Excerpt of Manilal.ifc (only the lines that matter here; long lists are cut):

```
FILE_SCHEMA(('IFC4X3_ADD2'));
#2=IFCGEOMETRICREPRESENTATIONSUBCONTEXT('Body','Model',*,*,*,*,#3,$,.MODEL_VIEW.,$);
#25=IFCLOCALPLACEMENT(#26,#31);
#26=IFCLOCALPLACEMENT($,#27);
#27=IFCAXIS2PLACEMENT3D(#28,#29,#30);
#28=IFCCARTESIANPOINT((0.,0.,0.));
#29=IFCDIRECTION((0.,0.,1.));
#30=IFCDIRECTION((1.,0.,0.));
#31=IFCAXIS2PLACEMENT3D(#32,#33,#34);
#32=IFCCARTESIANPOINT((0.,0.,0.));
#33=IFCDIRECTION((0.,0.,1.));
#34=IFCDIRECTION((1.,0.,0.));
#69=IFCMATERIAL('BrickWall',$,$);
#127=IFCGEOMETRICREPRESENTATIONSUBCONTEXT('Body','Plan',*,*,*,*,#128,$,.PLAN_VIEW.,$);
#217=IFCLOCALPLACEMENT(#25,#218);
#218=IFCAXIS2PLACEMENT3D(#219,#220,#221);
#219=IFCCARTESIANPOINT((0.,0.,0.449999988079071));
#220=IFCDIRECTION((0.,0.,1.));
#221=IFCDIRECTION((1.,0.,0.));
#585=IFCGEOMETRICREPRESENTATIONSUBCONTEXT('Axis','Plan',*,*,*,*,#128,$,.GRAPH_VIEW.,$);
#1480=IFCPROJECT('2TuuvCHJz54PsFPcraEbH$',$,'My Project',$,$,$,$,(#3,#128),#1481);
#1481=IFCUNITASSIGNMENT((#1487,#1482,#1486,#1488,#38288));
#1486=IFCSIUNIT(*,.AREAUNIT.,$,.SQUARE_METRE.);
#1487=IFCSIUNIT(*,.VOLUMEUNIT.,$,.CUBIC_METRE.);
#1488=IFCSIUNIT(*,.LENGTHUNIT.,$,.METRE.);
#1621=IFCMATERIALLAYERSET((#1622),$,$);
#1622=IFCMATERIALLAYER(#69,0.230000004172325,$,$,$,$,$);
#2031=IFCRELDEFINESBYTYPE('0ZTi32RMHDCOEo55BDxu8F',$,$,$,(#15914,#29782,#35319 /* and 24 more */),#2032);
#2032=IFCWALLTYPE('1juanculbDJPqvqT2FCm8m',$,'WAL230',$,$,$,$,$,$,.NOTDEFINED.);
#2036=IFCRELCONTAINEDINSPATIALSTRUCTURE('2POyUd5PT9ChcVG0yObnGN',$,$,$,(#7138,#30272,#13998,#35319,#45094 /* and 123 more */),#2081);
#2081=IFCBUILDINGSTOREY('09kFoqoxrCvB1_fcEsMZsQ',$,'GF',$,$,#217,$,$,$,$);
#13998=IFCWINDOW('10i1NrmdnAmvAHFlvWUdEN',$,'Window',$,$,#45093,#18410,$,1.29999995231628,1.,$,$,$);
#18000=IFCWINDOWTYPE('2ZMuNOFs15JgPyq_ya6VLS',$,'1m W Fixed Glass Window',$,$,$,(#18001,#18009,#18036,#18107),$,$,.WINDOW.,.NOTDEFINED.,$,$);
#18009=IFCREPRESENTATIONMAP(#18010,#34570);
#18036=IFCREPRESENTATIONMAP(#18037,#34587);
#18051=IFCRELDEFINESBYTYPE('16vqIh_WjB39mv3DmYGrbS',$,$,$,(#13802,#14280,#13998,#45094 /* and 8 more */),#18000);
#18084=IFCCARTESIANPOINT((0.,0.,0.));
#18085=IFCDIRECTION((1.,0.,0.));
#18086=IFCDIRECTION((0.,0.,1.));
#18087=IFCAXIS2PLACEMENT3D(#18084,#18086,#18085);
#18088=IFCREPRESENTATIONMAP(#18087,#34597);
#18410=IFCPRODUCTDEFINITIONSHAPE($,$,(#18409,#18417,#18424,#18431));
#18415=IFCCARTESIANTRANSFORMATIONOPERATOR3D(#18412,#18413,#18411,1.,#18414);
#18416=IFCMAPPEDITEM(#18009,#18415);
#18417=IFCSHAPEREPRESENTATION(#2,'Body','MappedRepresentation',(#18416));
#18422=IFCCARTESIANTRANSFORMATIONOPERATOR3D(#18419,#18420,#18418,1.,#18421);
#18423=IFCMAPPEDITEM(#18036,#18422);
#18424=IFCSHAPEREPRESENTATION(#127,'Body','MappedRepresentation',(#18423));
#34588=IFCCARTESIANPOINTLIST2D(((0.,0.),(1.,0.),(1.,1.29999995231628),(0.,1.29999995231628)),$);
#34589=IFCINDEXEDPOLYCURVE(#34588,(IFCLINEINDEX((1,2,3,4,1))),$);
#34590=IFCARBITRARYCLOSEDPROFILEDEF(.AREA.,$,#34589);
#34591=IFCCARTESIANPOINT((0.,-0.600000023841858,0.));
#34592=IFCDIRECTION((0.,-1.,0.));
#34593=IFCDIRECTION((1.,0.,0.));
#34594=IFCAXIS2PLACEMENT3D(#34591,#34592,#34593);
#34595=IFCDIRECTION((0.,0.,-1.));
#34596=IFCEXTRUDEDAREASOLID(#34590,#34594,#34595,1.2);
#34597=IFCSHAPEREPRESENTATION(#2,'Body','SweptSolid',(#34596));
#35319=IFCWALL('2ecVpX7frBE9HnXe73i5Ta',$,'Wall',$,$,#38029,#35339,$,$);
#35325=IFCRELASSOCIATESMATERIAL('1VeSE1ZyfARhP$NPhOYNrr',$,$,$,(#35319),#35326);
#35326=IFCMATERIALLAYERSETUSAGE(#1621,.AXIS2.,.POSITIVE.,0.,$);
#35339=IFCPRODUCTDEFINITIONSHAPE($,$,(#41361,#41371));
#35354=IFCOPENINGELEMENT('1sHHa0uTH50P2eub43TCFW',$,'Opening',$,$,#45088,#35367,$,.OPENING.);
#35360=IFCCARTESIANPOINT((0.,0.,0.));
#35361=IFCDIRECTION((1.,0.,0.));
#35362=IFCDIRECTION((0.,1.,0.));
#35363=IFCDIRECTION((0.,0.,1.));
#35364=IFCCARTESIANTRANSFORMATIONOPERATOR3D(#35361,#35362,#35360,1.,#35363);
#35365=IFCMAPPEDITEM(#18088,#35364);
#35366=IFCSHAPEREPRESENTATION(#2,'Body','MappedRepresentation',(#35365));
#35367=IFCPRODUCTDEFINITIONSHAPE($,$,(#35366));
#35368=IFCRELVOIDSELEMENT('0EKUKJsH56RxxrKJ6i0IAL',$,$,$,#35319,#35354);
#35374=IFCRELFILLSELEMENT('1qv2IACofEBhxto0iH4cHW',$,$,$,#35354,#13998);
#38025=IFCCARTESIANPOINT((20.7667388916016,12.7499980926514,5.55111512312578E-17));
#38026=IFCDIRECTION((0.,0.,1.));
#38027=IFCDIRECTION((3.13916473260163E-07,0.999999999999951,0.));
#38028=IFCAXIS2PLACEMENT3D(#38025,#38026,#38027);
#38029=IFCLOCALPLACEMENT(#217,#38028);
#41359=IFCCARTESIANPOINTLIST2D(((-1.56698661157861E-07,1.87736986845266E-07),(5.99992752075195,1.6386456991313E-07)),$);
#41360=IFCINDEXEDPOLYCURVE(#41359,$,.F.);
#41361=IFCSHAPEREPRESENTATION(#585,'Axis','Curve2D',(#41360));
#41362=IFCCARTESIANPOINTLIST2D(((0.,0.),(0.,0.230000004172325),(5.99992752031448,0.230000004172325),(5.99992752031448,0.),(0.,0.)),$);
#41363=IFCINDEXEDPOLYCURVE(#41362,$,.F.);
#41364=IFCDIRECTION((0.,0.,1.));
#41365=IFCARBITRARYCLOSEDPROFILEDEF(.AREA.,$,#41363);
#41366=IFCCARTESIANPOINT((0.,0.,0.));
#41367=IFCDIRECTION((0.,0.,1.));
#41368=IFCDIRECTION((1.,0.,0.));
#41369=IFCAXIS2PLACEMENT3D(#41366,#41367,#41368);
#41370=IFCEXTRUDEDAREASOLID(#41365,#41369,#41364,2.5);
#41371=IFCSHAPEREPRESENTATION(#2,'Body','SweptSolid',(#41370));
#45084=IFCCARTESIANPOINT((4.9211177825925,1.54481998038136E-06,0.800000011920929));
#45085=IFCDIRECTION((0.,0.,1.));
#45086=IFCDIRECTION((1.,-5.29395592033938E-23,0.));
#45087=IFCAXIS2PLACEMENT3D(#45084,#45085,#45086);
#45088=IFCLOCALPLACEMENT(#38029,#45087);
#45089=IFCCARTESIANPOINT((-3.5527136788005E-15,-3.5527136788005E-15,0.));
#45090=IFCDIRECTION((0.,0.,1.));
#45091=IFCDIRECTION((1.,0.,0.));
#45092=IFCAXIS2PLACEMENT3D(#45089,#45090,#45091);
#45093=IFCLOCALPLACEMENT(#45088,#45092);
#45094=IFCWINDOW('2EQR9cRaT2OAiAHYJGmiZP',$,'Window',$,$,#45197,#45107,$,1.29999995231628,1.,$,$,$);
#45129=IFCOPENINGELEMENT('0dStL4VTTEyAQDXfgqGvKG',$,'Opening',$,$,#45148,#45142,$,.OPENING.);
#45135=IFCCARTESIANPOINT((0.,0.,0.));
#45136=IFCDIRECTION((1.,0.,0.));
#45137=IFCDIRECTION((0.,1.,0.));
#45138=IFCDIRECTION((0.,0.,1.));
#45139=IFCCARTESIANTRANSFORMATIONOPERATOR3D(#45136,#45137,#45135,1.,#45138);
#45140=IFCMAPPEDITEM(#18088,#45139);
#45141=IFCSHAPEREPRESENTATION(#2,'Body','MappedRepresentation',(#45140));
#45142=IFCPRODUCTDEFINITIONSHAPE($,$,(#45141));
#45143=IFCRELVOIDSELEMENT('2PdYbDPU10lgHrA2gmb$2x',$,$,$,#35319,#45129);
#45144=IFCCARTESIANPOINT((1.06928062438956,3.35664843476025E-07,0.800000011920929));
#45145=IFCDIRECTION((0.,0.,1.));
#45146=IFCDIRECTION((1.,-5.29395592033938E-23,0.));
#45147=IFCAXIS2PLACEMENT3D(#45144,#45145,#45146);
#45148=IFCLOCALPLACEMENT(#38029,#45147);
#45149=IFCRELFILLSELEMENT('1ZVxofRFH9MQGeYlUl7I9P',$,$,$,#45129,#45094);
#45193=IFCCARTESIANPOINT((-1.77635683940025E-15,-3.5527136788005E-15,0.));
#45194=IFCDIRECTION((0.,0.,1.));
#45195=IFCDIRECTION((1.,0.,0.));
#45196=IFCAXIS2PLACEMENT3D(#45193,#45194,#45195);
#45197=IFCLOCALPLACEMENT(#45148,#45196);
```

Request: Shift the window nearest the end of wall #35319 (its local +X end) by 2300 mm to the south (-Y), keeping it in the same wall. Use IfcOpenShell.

```python
import ifcopenshell
import ifcopenshell.api.geometry
import ifcopenshell.util.placement

model = ifcopenshell.open("Manilal.ifc")

window = model.by_guid("10i1NrmdnAmvAHFlvWUdEN")
opening = window.FillsVoids[0].RelatingOpeningElement
wall = opening.VoidsElements[0].RelatingBuildingElement

wall_matrix = ifcopenshell.util.placement.get_local_placement(wall.ObjectPlacement)
shift = wall_matrix[:3, 0] * -2.3
before = ifcopenshell.util.placement.get_local_placement(window.ObjectPlacement)[:3, 3].copy()

# The window is placed relative to its opening, so it follows when the opening moves.
matrix = ifcopenshell.util.placement.get_local_placement(opening.ObjectPlacement)
matrix[:3, 3] += shift
ifcopenshell.api.geometry.edit_object_placement(
    model, product=opening, matrix=matrix, is_si=False, should_transform_children=True
)

after = ifcopenshell.util.placement.get_local_placement(window.ObjectPlacement)[:3, 3]
print("window moved by", (after - before).round(3) + 0.0)

model.write("Manilal_updated.ifc")
```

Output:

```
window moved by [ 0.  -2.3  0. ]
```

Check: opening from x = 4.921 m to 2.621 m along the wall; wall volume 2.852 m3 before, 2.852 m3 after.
